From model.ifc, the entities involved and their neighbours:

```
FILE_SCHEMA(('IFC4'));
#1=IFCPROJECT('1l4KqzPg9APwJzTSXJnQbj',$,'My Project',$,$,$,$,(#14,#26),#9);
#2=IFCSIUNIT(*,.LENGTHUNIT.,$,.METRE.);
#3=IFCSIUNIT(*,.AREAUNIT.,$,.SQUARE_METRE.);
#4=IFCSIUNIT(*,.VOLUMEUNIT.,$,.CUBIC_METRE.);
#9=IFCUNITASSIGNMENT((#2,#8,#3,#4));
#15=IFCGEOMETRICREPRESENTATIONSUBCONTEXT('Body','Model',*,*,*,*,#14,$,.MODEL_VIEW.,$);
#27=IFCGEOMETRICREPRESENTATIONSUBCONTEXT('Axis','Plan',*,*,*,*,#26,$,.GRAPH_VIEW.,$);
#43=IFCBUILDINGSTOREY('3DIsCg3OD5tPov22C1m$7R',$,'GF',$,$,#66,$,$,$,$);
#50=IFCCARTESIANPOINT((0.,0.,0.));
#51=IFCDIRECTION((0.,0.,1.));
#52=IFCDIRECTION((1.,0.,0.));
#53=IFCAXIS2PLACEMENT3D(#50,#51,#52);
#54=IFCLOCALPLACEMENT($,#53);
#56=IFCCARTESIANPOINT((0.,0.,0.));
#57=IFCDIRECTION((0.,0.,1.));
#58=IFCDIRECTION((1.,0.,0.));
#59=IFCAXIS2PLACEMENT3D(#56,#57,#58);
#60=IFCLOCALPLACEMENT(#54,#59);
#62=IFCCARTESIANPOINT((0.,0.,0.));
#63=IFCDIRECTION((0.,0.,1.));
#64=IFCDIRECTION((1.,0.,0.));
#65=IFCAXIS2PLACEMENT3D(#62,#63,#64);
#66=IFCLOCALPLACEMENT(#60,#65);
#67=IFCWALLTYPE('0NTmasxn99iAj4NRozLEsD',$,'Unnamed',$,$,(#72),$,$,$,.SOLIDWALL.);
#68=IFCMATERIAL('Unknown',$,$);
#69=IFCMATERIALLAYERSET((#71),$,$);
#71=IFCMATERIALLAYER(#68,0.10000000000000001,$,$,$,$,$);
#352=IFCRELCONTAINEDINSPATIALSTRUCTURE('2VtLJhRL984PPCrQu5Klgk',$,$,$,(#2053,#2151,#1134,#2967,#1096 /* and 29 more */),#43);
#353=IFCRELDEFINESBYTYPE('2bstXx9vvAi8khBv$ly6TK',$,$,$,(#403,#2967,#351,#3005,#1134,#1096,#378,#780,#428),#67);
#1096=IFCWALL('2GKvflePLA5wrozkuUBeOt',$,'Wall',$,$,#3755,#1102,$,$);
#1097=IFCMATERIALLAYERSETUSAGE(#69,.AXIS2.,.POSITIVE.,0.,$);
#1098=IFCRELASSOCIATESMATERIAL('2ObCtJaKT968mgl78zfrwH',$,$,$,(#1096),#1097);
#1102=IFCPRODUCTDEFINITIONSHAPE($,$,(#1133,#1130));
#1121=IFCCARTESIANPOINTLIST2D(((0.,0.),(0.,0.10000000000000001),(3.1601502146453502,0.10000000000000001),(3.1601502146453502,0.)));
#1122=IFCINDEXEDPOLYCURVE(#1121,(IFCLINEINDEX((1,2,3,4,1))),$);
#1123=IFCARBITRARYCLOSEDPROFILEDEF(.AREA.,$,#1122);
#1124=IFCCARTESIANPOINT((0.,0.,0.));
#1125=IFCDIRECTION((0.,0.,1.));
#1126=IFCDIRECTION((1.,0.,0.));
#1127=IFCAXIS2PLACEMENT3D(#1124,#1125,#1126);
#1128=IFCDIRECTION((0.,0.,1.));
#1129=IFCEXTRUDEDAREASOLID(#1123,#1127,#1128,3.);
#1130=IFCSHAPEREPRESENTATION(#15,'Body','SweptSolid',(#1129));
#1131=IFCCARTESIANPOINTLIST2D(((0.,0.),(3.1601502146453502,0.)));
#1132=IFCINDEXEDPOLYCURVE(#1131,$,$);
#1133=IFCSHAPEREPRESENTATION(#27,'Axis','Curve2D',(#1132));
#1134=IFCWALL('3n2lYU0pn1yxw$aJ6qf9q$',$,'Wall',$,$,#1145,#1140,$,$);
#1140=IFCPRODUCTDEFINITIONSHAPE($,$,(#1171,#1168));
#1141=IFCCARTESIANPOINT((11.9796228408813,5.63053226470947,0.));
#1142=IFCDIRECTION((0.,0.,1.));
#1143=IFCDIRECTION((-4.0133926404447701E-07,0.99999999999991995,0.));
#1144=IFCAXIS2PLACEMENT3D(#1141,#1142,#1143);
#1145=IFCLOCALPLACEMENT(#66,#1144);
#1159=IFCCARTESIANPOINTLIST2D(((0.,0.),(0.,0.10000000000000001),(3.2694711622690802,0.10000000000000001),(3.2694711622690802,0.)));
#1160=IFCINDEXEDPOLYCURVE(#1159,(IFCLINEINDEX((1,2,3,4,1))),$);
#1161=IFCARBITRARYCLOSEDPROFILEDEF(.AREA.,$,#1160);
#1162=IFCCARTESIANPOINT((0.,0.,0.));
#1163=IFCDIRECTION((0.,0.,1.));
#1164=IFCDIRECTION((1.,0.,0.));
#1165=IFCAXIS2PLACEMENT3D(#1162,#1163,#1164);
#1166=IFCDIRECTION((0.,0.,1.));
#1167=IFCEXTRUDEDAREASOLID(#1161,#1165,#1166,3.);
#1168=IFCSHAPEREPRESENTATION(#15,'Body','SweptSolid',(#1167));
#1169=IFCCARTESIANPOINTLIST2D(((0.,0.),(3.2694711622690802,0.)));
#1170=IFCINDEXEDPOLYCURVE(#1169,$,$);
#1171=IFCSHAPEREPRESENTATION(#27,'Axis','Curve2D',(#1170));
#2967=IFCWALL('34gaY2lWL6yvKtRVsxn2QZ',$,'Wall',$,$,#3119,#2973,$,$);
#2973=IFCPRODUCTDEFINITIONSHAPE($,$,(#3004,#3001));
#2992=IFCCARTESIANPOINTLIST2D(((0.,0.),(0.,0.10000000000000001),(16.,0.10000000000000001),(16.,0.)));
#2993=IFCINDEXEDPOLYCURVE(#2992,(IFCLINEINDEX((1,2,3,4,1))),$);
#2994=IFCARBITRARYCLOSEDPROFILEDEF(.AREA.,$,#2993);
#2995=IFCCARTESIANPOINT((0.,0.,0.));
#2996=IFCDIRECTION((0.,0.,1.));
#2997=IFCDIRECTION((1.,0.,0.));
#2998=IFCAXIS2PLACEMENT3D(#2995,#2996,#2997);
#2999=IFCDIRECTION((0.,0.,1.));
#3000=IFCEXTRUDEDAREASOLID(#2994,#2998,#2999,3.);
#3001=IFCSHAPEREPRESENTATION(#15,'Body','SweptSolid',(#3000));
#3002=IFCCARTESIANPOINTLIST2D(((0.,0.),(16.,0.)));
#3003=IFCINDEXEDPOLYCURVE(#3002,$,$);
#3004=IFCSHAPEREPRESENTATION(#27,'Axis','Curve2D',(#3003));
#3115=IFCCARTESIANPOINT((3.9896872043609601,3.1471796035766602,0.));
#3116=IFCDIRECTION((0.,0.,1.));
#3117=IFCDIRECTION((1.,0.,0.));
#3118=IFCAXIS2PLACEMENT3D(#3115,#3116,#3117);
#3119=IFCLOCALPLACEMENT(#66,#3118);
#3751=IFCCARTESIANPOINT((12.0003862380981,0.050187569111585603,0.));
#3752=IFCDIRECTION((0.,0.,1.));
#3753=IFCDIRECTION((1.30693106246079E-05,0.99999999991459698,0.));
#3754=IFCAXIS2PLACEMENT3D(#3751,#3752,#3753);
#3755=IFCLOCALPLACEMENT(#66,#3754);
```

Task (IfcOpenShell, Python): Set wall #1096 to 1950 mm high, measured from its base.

```python
import ifcopenshell
import ifcopenshell.geom
import ifcopenshell.util.representation
import ifcopenshell.util.shape

model = ifcopenshell.open("model.ifc")
settings = ifcopenshell.geom.settings()


def volume(element):
    """Net volume in cubic metres, openings subtracted."""
    shape = ifcopenshell.geom.create_shape(settings, element)
    return ifcopenshell.util.shape.get_volume(shape.geometry)


wall = model.by_guid("2GKvflePLA5wrozkuUBeOt")
before = volume(wall)

body = ifcopenshell.util.representation.get_representation(wall, "Model", "Body")
solid = body.Items[0]
old_height = solid.Depth
solid.Depth = 1.95
after = volume(wall)

print(f"height {old_height:g} -> {solid.Depth:g}, volume {before:.3f} -> {after:.3f} m3")

model.write("model_v2.ifc")
```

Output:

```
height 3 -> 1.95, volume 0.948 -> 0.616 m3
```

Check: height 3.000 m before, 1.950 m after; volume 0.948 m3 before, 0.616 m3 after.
